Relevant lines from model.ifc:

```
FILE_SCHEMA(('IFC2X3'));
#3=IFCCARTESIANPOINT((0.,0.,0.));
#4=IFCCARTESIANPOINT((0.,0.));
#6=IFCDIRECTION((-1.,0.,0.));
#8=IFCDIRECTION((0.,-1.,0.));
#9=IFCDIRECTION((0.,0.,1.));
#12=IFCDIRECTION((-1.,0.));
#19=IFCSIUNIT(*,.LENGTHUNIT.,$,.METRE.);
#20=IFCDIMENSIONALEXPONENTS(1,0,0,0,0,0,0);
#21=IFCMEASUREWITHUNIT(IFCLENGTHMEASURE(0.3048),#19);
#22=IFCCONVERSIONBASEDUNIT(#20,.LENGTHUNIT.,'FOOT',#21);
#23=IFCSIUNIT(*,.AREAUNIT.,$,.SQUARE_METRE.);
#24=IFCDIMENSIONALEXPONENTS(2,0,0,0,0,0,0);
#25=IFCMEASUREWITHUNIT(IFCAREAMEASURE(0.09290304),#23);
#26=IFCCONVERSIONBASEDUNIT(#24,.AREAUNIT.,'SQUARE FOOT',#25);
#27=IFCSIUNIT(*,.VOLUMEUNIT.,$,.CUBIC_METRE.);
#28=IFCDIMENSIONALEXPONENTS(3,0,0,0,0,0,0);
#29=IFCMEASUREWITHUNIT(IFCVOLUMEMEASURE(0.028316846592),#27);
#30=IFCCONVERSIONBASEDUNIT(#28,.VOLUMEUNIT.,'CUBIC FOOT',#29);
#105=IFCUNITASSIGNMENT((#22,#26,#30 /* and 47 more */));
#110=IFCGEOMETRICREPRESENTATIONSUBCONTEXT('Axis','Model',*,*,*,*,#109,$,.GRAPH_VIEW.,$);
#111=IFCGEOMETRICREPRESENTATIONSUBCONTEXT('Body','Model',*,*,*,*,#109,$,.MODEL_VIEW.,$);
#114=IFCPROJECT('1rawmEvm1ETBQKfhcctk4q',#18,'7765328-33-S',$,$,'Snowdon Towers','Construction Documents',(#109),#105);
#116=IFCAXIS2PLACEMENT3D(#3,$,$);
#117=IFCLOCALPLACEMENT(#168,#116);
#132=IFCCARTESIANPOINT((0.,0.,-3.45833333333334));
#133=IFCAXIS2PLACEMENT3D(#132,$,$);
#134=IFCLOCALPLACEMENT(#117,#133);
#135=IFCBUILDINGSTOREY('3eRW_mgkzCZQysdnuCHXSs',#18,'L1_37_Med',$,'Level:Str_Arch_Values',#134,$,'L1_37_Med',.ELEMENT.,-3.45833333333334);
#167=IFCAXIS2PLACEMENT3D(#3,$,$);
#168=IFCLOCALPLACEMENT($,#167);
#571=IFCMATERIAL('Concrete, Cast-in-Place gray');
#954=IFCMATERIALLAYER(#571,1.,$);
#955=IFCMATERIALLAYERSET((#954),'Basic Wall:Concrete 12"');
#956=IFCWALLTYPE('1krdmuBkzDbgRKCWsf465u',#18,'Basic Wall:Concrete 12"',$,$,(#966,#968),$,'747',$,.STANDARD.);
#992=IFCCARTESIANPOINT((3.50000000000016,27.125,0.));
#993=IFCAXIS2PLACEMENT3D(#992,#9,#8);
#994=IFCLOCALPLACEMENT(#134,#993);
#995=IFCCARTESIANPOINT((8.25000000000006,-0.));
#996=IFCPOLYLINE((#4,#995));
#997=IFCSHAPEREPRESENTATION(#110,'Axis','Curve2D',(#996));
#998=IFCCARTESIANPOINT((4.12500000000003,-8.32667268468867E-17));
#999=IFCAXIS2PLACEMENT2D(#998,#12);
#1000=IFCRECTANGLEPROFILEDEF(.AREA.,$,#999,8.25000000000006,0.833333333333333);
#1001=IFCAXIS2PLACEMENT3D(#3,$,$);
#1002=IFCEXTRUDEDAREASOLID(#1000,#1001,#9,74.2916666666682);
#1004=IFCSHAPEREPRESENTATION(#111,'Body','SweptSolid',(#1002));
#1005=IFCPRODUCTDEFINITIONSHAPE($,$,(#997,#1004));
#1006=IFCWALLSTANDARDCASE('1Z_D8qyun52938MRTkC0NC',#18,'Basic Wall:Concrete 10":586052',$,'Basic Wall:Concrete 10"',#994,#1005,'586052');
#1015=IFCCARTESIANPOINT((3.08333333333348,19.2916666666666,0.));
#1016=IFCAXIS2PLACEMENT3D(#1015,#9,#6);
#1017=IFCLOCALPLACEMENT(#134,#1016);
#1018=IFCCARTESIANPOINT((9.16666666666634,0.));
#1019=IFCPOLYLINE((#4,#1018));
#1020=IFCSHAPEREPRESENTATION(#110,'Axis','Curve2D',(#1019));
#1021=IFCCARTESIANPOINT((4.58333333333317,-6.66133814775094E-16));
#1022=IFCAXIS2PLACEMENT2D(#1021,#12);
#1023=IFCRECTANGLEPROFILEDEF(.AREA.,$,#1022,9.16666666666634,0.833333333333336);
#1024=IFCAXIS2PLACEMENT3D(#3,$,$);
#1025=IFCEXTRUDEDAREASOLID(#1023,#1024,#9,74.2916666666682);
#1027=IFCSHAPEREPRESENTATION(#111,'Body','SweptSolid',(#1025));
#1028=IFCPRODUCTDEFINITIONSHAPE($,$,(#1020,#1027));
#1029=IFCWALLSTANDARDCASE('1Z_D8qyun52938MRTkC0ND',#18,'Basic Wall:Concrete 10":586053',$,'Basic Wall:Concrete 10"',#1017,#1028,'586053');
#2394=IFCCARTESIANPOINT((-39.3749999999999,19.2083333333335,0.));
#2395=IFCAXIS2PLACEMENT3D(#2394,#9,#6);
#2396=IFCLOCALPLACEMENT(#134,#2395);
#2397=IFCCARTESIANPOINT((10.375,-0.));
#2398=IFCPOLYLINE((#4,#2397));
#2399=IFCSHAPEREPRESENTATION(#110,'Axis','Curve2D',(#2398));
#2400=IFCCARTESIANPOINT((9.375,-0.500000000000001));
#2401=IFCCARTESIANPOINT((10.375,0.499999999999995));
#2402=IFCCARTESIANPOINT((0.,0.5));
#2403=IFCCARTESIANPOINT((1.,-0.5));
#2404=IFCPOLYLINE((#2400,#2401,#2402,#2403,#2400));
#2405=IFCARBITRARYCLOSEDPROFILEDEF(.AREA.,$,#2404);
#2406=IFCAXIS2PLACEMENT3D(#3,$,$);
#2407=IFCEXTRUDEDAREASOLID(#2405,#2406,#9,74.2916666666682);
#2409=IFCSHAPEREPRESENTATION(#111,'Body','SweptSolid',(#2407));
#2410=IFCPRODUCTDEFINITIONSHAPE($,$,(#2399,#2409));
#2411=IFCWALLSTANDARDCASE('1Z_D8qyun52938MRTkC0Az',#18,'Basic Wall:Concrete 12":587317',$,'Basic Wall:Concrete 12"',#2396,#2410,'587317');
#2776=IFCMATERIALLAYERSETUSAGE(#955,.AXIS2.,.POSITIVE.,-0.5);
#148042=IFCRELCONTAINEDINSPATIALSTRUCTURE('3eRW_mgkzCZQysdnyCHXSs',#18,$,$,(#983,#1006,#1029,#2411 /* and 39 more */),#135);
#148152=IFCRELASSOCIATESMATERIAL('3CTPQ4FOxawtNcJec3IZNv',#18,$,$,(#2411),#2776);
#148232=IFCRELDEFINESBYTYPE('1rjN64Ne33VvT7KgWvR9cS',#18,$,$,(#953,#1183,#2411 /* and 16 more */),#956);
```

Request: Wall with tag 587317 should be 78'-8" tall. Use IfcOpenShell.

```python
import ifcopenshell
import ifcopenshell.geom
import ifcopenshell.util.representation
import ifcopenshell.util.shape
import ifcopenshell.util.unit

model = ifcopenshell.open("model.ifc")
unit_scale = ifcopenshell.util.unit.calculate_unit_scale(model)
settings = ifcopenshell.geom.settings()


def volume(element):
    """Net volume in cubic metres, openings subtracted."""
    shape = ifcopenshell.geom.create_shape(settings, element)
    return ifcopenshell.util.shape.get_volume(shape.geometry)


wall = model.by_guid("1Z_D8qyun52938MRTkC0Az")
before = volume(wall)

body = ifcopenshell.util.representation.get_representation(wall, "Model", "Body")
solid = body.Items[0]
old_height = solid.Depth
solid.Depth = 944 * 0.0254 / unit_scale
after = volume(wall)

print(f"height {old_height:g} -> {solid.Depth:g}, volume {before:.3f} -> {after:.3f} m3")

model.write("model_updated.ifc")
```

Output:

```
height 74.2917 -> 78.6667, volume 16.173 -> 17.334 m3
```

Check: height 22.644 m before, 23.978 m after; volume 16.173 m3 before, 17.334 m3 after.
